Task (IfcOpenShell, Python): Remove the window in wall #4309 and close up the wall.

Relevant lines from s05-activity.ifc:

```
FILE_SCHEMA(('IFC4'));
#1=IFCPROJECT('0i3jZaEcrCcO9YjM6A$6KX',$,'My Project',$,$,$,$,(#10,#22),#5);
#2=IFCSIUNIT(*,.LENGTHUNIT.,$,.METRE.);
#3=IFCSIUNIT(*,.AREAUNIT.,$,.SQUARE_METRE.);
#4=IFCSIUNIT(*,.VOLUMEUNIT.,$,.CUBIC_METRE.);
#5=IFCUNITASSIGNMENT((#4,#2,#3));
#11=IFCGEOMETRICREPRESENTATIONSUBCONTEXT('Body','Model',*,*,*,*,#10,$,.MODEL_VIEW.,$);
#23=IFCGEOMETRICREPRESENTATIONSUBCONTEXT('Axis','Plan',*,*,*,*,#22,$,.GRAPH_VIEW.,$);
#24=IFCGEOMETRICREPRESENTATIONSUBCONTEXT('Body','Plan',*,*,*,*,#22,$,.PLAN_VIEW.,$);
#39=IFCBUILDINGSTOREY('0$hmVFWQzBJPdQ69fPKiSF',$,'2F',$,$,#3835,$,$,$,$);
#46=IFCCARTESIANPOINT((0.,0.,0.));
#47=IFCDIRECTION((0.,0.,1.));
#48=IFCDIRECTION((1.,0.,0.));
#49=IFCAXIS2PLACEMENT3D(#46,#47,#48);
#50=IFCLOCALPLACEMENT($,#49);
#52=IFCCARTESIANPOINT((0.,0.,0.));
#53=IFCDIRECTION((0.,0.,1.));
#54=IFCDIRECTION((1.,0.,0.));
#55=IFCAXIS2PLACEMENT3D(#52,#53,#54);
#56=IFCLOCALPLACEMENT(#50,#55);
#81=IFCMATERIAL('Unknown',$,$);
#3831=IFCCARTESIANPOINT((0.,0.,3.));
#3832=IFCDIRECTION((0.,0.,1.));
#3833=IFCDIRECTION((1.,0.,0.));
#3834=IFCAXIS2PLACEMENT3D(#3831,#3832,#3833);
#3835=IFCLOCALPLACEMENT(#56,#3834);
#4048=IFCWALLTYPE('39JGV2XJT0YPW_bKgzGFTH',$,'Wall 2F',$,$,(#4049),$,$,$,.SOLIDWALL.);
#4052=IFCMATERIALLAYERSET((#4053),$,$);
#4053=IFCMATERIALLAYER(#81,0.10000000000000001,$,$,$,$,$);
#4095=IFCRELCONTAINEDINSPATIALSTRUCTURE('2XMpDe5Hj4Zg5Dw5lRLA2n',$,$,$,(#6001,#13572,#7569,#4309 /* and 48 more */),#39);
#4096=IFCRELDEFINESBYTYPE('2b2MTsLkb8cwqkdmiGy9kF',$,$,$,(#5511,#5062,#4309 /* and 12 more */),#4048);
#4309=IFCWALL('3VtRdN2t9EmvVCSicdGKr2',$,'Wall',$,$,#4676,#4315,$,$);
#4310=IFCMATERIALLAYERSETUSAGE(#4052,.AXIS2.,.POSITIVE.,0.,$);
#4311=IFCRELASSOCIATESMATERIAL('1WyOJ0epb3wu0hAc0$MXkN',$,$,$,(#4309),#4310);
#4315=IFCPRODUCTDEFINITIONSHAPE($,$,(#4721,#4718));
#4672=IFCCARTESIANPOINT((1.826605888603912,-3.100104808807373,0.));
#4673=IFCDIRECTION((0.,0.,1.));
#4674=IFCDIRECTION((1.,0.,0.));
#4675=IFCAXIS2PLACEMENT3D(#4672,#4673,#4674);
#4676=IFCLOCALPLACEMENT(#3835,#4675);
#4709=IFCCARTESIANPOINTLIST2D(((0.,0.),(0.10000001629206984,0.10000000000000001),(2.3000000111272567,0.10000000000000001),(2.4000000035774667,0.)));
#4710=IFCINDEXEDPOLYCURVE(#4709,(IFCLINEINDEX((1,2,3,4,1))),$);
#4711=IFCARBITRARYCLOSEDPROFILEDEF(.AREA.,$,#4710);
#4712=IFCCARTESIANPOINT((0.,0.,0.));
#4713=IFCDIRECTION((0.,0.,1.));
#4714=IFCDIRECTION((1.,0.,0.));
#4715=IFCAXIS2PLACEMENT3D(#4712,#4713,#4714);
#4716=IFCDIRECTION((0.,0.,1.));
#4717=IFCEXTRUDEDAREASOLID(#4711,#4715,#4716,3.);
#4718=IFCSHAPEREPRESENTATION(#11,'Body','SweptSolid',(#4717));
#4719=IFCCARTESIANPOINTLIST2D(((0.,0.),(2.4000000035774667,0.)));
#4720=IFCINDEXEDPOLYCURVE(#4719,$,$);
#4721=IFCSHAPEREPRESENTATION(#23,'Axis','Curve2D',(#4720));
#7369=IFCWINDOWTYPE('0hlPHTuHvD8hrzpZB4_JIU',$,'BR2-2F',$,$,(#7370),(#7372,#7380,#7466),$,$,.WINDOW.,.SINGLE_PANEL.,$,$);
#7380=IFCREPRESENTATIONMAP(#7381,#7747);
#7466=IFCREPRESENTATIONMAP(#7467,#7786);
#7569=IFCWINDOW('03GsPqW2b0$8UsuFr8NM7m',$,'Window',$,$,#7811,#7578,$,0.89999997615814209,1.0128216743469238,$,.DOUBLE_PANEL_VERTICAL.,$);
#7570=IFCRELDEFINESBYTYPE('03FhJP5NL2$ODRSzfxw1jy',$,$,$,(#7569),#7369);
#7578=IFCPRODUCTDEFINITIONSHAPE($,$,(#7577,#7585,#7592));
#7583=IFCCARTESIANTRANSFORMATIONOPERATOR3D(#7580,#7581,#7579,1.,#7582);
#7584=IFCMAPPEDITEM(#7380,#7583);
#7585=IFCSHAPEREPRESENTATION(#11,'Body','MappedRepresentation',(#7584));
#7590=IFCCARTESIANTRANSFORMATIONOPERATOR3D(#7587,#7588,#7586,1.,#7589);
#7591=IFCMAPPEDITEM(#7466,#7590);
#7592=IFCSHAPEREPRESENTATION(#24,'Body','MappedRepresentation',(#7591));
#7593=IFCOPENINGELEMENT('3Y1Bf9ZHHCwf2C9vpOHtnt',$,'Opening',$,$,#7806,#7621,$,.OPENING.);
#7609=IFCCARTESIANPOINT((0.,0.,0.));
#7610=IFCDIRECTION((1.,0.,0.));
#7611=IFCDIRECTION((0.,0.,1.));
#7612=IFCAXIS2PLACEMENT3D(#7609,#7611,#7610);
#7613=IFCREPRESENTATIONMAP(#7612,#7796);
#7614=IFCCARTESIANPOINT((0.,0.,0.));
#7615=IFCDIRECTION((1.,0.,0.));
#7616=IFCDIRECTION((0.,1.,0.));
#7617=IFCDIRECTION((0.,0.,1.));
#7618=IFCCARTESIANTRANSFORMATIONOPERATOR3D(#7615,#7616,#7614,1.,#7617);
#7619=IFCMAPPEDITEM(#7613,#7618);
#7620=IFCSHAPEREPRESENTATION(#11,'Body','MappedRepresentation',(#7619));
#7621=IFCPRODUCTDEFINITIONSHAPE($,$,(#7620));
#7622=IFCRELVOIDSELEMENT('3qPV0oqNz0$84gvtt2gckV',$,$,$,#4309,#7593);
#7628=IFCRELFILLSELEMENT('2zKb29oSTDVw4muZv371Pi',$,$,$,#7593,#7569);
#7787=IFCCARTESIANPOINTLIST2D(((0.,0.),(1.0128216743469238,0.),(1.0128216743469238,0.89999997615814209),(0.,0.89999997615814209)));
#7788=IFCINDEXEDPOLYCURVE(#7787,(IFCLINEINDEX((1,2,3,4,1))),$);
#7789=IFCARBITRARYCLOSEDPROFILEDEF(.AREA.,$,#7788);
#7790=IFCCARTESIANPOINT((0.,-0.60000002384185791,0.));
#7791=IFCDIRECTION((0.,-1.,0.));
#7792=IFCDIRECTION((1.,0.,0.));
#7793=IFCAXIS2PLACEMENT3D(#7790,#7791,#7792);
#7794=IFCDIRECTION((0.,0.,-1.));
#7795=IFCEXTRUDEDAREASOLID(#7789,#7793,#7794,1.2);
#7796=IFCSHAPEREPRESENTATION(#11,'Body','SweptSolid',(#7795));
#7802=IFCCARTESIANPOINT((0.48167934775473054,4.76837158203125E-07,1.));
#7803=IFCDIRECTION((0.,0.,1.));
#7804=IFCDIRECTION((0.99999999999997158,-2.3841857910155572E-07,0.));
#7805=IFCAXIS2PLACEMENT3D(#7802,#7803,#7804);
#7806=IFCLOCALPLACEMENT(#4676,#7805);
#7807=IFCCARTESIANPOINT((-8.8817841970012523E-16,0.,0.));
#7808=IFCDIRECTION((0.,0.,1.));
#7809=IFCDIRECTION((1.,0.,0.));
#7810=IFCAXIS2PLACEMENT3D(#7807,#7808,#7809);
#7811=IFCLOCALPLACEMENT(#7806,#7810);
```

```python
import ifcopenshell
import ifcopenshell.api.feature
import ifcopenshell.api.root
import ifcopenshell.geom
import ifcopenshell.util.shape

model = ifcopenshell.open("s05-activity.ifc")
settings = ifcopenshell.geom.settings()


def volume(element):
    """Net volume in cubic metres, openings subtracted."""
    shape = ifcopenshell.geom.create_shape(settings, element)
    return ifcopenshell.util.shape.get_volume(shape.geometry)


window = model.by_guid("03GsPqW2b0$8UsuFr8NM7m")
opening = window.FillsVoids[0].RelatingOpeningElement
wall = opening.VoidsElements[0].RelatingBuildingElement
before = volume(wall)

ifcopenshell.api.root.remove_product(model, product=window)
ifcopenshell.api.feature.remove_feature(model, feature=opening)

after = volume(wall)

print(f"wall volume {before:.3f} -> {after:.3f} m3")

model.write("s05-activity-out.ifc")
```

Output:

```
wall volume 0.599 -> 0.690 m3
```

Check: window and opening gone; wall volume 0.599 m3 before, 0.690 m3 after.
